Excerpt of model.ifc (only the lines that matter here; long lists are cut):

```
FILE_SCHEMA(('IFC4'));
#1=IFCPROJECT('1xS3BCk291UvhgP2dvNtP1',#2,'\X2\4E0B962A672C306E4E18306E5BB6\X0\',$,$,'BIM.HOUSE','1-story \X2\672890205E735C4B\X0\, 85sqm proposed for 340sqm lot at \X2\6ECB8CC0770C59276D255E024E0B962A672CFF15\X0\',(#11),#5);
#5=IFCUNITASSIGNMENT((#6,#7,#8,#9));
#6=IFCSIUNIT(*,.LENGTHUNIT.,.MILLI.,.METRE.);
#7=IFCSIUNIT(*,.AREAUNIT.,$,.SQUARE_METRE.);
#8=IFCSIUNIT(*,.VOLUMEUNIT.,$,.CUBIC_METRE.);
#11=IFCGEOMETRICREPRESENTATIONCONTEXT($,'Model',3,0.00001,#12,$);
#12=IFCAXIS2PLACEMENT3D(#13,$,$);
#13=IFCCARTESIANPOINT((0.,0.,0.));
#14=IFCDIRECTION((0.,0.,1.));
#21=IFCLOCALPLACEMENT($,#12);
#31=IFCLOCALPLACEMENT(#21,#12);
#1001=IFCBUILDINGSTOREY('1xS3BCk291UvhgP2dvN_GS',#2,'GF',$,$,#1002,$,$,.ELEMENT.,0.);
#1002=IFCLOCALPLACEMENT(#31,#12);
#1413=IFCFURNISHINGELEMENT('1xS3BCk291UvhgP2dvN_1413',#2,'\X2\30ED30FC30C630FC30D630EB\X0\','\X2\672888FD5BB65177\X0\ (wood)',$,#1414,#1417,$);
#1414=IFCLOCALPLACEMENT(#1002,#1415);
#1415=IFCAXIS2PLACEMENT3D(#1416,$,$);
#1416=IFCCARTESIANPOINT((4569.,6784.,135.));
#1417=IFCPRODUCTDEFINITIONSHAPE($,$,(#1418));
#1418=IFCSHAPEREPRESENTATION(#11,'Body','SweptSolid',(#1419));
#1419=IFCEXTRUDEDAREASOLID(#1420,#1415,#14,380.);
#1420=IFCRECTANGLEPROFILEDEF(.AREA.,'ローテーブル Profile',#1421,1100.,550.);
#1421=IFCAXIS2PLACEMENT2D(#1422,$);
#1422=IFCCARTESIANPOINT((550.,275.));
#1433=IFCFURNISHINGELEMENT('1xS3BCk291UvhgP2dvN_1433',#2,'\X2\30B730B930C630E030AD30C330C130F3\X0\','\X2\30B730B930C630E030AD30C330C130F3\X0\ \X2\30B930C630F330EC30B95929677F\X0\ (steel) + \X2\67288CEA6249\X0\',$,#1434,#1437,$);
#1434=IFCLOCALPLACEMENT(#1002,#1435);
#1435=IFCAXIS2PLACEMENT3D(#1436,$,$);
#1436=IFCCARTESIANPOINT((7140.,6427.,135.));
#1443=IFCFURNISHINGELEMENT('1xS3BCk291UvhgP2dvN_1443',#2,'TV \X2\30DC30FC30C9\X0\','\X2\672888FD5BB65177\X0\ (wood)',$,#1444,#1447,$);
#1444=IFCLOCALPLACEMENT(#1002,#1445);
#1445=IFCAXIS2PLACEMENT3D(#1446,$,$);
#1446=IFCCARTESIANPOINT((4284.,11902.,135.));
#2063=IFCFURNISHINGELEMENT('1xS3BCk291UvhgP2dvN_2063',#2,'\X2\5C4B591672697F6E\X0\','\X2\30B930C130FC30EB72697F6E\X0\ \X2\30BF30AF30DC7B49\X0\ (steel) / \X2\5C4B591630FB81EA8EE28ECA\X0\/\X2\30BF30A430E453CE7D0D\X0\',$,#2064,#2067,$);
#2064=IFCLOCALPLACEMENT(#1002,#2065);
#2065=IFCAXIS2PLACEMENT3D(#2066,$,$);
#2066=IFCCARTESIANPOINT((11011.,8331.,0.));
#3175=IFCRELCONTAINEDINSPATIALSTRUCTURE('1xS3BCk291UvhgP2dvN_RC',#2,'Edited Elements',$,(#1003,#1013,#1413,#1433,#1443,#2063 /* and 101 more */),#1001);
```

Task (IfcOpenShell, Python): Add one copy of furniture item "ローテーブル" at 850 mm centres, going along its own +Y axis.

```python
import ifcopenshell
import ifcopenshell.api.geometry
import ifcopenshell.api.root
import ifcopenshell.util.element
import ifcopenshell.util.placement

model = ifcopenshell.open("model.ifc")


def reuse_history(source, copy):
    """copy_class also copies each property set's owner history, people and application; keep the originals."""
    for rel in copy.IsDefinedBy:
        if rel.is_a("IfcRelDefinesByProperties") and (history := rel.RelatingPropertyDefinition.OwnerHistory):
            rel.RelatingPropertyDefinition.OwnerHistory = source.OwnerHistory
            ifcopenshell.util.element.remove_deep2(model, history)


source = model.by_guid("1xS3BCk291UvhgP2dvN_1413")
base = ifcopenshell.util.placement.get_local_placement(source.ObjectPlacement)
step = base[:3, 1] * 850.0

for i in range(1, 2):
    copy = ifcopenshell.api.root.copy_class(model, product=source)
    copy.Representation = ifcopenshell.util.element.copy_deep(
        model, source.Representation, exclude=["IfcGeometricRepresentationContext", "IfcRepresentationMap"]
    )
    reuse_history(source, copy)
    matrix = base.copy()
    matrix[:3, 3] += i * step
    print("added at", matrix[:3, 3].round(3) + 0.0)
    ifcopenshell.api.geometry.edit_object_placement(model, product=copy, matrix=matrix, is_si=False)

model.write("model_v2.ifc")
```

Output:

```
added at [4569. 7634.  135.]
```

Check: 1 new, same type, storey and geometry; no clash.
